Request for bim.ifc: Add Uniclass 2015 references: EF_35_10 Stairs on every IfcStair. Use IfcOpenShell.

First a look at what the model holds.

```python
import ifcopenshell

model = ifcopenshell.open("bim.ifc")
print(model.schema)
print("classifications:", [c.Name for c in model.by_type("IfcClassification")])
for ifc_class in ("IfcDoor", "IfcRoof", "IfcStair", "IfcWall", "IfcWindow"):
    print(ifc_class, len(model.by_type(ifc_class)))
```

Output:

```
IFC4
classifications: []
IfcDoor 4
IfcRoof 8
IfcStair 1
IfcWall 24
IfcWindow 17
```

```python
import ifcopenshell
import ifcopenshell.api.classification

model = ifcopenshell.open("bim.ifc")

system = ifcopenshell.api.classification.add_classification(model, classification="Uniclass 2015")

codes = {
    "IfcStair": ("EF_35_10", "Stairs"),
}
for ifc_class, (code, name) in codes.items():
    products = model.by_type(ifc_class)
    ifcopenshell.api.classification.add_reference(
        model, products=products, classification=system, identification=code, name=name
    )
    print(code, len(products))

model.write("bim-out.ifc")
```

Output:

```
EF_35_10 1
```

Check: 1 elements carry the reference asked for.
